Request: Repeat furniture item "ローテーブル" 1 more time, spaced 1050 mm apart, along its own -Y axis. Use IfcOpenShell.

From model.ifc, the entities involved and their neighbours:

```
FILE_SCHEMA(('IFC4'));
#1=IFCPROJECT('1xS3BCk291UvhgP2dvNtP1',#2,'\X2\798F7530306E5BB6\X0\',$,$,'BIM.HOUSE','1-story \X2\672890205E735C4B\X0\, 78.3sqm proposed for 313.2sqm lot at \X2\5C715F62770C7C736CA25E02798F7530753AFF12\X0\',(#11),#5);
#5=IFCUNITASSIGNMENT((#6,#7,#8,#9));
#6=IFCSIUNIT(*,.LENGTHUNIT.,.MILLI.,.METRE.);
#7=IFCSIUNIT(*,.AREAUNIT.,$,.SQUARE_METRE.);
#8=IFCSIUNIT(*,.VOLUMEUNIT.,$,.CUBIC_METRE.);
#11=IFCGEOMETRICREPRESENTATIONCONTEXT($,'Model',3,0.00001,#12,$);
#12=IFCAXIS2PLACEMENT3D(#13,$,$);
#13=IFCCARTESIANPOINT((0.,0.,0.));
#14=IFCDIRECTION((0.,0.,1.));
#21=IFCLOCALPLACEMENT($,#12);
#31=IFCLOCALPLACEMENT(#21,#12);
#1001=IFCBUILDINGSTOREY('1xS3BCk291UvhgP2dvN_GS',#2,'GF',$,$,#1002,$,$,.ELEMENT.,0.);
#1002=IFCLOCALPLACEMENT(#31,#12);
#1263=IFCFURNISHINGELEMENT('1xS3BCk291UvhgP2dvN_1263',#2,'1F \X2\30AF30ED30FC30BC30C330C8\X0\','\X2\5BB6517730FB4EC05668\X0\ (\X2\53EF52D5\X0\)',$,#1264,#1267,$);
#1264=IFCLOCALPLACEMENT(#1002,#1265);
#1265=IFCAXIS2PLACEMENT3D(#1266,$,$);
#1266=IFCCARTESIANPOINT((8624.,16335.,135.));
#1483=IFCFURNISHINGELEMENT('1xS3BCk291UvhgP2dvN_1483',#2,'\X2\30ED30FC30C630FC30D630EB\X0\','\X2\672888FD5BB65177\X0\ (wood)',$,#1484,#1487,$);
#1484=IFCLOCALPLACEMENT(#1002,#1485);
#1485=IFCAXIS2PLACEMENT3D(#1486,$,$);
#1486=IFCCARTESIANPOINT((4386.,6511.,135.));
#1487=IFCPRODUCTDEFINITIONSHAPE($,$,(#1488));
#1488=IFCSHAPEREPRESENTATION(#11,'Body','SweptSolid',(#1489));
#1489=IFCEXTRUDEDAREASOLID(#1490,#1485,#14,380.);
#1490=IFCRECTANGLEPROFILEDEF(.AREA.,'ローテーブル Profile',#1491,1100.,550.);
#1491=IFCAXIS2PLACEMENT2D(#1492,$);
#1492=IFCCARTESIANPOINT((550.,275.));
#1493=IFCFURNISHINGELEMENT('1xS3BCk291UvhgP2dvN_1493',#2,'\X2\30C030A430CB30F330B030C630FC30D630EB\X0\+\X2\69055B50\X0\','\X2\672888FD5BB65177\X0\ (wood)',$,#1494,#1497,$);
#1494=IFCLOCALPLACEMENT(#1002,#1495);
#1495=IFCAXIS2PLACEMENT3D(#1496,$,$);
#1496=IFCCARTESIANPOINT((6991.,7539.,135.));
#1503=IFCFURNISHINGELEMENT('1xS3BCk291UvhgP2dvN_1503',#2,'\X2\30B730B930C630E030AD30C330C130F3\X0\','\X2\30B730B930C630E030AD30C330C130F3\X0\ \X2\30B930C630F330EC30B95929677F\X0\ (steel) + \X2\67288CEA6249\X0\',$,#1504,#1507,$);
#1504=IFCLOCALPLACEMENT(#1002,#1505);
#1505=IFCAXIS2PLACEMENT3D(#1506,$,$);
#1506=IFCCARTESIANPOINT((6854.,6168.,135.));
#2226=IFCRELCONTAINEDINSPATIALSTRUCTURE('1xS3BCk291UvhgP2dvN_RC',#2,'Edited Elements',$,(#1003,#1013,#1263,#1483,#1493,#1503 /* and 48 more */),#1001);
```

```python
import ifcopenshell
import ifcopenshell.api.geometry
import ifcopenshell.api.root
import ifcopenshell.util.element
import ifcopenshell.util.placement

model = ifcopenshell.open("model.ifc")


def reuse_history(source, copy):
    """copy_class also copies each property set's owner history, people and application; keep the originals."""
    for rel in copy.IsDefinedBy:
        if rel.is_a("IfcRelDefinesByProperties") and (history := rel.RelatingPropertyDefinition.OwnerHistory):
            rel.RelatingPropertyDefinition.OwnerHistory = source.OwnerHistory
            ifcopenshell.util.element.remove_deep2(model, history)


source = model.by_id(1483)
base = ifcopenshell.util.placement.get_local_placement(source.ObjectPlacement)
step = -base[:3, 1] * 1050.0

for i in range(1, 2):
    copy = ifcopenshell.api.root.copy_class(model, product=source)
    copy.Representation = ifcopenshell.util.element.copy_deep(
        model, source.Representation, exclude=["IfcGeometricRepresentationContext", "IfcRepresentationMap"]
    )
    reuse_history(source, copy)
    matrix = base.copy()
    matrix[:3, 3] += i * step
    print("added at", matrix[:3, 3].round(3) + 0.0)
    ifcopenshell.api.geometry.edit_object_placement(model, product=copy, matrix=matrix, is_si=False)

model.write("model-out.ifc")
```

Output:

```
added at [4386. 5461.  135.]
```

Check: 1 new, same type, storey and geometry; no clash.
